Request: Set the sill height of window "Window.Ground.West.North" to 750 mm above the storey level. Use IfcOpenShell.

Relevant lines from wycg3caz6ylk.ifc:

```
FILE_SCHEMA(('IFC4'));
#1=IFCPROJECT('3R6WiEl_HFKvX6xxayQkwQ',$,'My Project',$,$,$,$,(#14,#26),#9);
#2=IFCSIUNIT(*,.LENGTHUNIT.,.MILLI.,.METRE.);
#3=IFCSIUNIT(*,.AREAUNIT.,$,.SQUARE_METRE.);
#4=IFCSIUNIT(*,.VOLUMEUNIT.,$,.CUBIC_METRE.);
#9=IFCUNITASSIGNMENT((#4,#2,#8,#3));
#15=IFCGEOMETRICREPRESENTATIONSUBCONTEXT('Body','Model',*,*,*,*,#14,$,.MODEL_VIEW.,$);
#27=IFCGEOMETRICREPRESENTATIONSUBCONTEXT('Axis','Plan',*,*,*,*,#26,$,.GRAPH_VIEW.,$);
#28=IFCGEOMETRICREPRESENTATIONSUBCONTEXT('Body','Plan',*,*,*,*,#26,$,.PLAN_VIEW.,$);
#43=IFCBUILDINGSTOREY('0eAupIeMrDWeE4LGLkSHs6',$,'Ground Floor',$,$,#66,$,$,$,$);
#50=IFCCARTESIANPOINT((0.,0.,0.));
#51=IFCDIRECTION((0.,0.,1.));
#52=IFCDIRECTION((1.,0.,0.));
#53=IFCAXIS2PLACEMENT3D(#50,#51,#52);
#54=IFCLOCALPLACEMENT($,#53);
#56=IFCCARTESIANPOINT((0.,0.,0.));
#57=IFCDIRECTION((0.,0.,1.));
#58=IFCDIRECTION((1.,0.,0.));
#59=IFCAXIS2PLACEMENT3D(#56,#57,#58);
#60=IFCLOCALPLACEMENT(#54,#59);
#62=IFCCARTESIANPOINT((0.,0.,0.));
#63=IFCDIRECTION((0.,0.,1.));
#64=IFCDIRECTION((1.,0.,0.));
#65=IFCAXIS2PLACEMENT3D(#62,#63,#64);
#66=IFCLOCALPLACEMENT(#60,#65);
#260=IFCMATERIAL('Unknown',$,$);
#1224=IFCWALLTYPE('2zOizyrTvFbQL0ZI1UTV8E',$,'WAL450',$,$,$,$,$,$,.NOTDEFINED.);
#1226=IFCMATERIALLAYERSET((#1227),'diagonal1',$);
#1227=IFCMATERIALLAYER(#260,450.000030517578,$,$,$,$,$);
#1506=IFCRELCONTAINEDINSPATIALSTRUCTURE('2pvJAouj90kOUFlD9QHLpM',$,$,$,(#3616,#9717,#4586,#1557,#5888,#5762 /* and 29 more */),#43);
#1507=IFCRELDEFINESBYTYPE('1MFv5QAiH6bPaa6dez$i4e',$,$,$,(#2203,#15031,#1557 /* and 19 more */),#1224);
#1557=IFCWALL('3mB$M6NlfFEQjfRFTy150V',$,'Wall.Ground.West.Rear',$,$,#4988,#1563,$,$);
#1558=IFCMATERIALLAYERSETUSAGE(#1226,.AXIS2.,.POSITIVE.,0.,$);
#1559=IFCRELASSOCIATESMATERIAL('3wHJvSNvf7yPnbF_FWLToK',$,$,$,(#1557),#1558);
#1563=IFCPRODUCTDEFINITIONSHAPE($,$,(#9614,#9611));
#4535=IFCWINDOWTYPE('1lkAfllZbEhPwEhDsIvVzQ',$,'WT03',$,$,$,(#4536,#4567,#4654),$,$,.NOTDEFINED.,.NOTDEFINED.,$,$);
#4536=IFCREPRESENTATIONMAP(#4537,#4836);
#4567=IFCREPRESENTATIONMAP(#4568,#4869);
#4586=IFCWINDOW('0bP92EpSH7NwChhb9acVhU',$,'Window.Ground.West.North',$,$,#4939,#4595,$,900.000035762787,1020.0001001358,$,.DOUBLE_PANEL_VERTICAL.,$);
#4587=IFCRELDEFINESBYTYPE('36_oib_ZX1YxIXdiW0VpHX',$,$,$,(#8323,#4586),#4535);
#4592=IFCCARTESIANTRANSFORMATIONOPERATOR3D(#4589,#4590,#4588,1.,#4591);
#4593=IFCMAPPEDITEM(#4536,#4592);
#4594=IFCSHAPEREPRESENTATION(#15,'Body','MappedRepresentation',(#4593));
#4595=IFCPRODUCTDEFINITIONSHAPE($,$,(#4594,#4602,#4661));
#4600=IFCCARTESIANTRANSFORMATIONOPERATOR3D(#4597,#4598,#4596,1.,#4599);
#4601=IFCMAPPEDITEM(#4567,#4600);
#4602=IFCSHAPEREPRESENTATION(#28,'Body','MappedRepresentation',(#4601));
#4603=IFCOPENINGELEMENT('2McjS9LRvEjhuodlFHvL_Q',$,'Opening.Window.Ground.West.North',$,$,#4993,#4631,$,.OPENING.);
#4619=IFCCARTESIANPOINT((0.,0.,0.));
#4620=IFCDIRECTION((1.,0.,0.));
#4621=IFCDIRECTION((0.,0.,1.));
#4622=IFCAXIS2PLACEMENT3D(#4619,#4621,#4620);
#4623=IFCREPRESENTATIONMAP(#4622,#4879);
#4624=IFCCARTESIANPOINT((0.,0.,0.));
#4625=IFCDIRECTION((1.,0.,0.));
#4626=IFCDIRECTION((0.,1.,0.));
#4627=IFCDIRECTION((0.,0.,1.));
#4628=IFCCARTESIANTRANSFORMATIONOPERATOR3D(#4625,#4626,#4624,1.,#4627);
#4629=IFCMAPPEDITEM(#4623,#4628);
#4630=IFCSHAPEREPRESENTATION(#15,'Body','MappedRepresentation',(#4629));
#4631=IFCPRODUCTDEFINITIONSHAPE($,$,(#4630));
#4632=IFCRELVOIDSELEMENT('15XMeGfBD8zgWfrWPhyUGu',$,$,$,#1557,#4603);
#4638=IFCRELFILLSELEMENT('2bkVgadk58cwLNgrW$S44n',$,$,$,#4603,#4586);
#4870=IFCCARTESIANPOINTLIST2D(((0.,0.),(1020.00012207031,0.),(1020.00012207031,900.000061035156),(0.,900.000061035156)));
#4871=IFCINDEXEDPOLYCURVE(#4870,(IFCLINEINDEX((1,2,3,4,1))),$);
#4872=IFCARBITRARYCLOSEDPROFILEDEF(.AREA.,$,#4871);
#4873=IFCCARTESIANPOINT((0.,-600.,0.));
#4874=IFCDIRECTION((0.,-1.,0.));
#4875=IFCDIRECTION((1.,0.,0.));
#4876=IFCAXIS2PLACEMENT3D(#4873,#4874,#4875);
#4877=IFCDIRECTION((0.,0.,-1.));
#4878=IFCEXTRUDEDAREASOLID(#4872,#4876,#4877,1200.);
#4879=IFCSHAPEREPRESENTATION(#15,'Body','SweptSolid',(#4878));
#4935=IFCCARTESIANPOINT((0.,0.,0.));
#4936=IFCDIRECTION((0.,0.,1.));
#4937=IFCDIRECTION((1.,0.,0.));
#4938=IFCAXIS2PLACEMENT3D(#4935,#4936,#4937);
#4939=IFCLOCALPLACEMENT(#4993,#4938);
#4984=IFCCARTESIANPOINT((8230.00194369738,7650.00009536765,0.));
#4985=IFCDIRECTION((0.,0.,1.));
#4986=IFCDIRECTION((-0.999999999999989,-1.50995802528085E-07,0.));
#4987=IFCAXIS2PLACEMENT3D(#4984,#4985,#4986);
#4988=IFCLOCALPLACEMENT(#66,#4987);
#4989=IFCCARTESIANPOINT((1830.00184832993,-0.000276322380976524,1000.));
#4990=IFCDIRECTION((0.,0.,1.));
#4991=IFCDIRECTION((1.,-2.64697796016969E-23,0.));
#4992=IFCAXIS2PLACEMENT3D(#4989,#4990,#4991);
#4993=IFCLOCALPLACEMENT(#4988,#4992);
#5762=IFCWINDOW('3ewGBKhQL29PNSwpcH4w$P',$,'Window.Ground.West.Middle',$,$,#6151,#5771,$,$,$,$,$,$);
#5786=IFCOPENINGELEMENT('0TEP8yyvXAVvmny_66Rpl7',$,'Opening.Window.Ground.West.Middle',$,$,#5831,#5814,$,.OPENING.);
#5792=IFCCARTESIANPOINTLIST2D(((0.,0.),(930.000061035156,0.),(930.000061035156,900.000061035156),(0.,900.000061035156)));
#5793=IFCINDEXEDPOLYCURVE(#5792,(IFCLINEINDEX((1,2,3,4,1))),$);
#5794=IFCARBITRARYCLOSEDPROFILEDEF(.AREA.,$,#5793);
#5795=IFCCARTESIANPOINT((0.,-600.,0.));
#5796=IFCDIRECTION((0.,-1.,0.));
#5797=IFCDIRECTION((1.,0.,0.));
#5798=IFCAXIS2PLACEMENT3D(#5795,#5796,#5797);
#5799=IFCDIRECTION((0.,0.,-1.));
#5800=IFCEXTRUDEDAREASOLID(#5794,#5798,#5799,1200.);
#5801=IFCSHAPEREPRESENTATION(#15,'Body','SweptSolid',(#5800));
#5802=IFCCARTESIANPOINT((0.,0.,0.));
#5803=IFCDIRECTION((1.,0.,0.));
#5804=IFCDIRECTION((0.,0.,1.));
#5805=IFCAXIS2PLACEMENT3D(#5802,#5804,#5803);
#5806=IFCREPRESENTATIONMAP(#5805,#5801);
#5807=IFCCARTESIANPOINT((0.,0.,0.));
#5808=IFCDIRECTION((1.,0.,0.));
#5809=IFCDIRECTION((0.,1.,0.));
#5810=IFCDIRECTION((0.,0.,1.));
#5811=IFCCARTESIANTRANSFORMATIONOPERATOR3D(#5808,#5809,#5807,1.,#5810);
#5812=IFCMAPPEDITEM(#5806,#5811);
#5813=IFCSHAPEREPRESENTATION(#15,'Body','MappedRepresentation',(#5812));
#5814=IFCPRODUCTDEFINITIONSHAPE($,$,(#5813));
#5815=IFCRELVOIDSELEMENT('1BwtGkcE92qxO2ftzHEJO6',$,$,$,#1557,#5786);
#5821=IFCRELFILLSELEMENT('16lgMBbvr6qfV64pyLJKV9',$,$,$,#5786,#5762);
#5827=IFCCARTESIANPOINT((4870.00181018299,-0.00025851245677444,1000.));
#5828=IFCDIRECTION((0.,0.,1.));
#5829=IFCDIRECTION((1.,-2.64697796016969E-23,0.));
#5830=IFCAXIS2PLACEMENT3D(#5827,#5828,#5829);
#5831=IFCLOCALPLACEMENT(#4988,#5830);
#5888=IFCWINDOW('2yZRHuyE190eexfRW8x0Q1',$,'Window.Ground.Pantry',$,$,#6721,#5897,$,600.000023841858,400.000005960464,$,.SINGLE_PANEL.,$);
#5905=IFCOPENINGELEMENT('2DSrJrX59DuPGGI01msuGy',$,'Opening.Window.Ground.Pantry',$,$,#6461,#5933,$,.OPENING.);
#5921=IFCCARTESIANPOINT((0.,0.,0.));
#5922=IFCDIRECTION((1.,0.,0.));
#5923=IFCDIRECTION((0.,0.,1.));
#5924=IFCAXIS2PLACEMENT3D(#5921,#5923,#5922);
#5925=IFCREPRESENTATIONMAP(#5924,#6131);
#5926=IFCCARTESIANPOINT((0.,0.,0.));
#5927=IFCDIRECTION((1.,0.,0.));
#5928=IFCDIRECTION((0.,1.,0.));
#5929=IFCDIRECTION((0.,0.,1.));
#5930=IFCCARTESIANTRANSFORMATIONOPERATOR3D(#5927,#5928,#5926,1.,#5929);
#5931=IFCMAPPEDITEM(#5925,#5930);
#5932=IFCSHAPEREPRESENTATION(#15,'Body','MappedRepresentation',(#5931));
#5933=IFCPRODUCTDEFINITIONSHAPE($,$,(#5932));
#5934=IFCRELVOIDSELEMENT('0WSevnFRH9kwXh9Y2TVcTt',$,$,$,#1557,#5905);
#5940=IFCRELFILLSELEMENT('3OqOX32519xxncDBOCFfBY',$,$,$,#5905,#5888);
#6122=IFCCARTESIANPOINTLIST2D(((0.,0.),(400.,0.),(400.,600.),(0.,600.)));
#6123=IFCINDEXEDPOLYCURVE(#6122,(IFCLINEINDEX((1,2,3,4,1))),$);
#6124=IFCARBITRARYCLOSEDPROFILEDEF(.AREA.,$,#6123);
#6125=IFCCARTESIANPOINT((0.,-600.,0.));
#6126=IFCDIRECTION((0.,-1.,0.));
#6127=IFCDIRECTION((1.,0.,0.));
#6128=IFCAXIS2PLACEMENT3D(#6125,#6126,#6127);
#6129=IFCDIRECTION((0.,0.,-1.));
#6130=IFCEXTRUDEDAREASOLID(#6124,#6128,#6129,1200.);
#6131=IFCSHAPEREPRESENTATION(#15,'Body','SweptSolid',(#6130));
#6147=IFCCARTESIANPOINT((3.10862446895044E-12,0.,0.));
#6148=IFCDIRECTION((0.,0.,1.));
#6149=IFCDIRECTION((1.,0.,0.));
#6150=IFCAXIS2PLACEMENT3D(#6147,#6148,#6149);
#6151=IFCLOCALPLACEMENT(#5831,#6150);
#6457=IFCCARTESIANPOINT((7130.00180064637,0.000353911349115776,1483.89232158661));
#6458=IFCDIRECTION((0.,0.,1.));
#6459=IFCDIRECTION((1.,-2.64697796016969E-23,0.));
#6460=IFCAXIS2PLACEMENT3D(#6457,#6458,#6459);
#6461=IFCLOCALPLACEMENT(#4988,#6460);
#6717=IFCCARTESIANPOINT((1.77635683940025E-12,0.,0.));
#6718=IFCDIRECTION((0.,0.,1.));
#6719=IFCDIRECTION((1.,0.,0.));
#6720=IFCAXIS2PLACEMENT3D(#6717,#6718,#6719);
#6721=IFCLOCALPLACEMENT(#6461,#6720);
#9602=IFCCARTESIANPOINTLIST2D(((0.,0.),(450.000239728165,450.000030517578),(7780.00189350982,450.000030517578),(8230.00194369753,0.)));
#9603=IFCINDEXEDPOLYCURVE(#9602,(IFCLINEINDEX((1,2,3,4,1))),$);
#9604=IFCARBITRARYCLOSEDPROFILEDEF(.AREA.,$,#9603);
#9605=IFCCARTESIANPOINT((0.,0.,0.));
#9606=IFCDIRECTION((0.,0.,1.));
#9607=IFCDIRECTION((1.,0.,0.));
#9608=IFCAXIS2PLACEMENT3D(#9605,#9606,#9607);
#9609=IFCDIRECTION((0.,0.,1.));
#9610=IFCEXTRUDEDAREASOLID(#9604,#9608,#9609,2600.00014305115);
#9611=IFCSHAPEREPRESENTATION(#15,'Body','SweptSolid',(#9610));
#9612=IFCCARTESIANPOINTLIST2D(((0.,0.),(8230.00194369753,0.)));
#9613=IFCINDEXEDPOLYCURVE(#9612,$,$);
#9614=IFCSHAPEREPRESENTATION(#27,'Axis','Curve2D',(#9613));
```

```python
import numpy as np
import ifcopenshell
import ifcopenshell.api.geometry
import ifcopenshell.geom
import ifcopenshell.util.element
import ifcopenshell.util.placement
import ifcopenshell.util.shape
import ifcopenshell.util.unit

model = ifcopenshell.open("wycg3caz6ylk.ifc")
unit_scale = ifcopenshell.util.unit.calculate_unit_scale(model)

window = model.by_guid("0bP92EpSH7NwChhb9acVhU")
opening = window.FillsVoids[0].RelatingOpeningElement
storey = ifcopenshell.util.element.get_container(window, ifc_class="IfcBuildingStorey")
level = ifcopenshell.util.placement.get_local_placement(storey.ObjectPlacement)[2, 3]

# The opening's origin need not be at the sill, so measure its lowest point.
shape = ifcopenshell.geom.create_shape(ifcopenshell.geom.settings(), opening)
bottom = ifcopenshell.util.shape.get_shape_bottom_elevation(shape, shape.geometry) / unit_scale
dz = level + 750.0 - bottom

shift = np.array([0.0, 0.0, dz])
# The window is placed relative to its opening, so it follows when the opening moves.
matrix = ifcopenshell.util.placement.get_local_placement(opening.ObjectPlacement)
matrix[:3, 3] += shift
ifcopenshell.api.geometry.edit_object_placement(
    model, product=opening, matrix=matrix, is_si=False, should_transform_children=True
)

print(f"moved by {dz * unit_scale:+.3f} m")

model.write("wycg3caz6ylk_v2.ifc")
```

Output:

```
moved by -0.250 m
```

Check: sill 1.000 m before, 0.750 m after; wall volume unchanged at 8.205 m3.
